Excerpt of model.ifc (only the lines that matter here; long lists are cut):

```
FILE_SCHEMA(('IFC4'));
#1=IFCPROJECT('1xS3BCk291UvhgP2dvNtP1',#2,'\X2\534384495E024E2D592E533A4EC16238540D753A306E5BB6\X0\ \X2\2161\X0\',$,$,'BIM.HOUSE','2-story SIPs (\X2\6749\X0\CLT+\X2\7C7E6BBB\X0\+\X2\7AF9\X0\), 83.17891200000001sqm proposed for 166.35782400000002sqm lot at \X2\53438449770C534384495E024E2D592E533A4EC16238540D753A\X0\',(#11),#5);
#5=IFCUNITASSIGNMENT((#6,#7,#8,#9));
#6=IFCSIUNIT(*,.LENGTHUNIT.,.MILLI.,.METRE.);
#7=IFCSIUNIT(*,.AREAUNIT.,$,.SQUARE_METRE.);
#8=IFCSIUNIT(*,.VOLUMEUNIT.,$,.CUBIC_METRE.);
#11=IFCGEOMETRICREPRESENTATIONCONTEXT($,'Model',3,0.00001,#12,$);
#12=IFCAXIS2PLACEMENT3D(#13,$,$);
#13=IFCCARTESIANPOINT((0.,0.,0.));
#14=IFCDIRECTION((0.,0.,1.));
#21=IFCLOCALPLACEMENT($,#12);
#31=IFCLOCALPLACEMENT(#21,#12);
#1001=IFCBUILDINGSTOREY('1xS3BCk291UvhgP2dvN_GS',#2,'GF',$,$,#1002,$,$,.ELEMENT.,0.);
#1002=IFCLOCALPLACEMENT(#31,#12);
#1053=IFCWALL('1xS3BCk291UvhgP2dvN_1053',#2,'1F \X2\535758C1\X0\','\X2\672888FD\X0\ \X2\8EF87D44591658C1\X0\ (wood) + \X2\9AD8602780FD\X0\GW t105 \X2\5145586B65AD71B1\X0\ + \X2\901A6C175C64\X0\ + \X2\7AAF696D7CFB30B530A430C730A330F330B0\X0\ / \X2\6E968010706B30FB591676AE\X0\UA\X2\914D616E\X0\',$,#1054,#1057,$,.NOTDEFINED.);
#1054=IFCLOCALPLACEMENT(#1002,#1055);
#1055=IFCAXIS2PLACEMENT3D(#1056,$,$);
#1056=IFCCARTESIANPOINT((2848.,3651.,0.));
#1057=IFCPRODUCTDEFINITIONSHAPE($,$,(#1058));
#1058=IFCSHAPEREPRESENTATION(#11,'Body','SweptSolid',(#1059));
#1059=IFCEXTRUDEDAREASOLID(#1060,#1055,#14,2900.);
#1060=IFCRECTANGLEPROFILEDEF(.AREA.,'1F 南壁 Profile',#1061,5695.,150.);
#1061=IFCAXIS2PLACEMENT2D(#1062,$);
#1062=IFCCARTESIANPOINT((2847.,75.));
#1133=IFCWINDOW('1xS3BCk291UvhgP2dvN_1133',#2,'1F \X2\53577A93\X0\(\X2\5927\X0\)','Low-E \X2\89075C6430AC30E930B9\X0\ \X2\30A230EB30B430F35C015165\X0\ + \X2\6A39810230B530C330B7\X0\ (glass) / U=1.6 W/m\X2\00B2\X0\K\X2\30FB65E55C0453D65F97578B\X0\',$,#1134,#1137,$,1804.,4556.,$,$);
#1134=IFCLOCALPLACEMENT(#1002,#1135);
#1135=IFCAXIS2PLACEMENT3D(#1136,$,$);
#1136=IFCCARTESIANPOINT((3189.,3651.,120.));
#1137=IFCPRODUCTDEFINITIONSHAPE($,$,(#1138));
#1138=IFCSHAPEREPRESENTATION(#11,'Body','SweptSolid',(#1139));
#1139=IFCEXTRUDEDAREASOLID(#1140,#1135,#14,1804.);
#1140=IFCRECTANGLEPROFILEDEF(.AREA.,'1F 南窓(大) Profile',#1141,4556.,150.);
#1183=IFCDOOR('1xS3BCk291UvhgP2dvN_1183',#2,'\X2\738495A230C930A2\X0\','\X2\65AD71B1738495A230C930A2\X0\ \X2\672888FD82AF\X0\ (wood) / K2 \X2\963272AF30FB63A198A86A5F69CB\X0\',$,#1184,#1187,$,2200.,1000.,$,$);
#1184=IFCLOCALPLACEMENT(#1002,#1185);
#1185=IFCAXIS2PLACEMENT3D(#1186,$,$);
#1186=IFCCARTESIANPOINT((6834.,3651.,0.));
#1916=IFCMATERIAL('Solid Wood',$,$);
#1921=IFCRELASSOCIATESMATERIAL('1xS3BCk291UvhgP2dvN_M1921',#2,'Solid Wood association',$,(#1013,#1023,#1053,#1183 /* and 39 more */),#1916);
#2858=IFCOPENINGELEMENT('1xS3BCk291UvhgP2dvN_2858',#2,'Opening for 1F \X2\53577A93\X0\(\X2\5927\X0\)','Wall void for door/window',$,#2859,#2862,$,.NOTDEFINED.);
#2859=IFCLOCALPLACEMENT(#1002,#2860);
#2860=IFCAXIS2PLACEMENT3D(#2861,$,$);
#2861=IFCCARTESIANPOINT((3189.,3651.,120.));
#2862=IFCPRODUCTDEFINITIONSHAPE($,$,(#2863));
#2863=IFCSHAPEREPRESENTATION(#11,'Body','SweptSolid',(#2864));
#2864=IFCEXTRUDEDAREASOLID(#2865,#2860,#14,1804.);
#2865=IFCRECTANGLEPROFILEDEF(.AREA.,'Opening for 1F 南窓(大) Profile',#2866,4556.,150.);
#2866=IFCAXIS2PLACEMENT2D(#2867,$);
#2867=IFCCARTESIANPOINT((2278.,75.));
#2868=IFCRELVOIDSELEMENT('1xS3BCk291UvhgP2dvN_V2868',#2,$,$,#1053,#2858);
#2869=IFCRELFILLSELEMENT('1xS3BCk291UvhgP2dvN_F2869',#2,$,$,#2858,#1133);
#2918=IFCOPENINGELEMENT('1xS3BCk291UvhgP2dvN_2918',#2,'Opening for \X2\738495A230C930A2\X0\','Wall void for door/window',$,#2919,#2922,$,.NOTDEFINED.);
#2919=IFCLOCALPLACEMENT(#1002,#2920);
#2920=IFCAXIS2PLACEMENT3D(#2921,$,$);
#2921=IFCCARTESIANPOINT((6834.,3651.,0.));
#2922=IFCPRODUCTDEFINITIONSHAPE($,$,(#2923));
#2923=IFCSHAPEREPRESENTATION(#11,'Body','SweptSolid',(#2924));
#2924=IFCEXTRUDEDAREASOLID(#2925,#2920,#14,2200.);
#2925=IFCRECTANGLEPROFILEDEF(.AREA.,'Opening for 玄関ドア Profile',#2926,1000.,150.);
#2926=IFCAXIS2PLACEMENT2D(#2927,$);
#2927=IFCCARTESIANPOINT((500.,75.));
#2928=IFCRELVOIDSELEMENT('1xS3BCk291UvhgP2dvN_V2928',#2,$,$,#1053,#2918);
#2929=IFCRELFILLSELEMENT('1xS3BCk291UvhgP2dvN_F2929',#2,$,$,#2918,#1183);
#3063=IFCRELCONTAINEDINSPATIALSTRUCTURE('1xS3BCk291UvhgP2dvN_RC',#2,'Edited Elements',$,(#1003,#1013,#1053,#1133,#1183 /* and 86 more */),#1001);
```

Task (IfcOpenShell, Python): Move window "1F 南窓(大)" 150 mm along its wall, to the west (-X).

```python
import ifcopenshell
import ifcopenshell.api.geometry
import ifcopenshell.util.placement
import ifcopenshell.util.unit

model = ifcopenshell.open("model.ifc")
unit_scale = ifcopenshell.util.unit.calculate_unit_scale(model)

window = model.by_guid("1xS3BCk291UvhgP2dvN_1133")
opening = window.FillsVoids[0].RelatingOpeningElement
wall = opening.VoidsElements[0].RelatingBuildingElement

wall_matrix = ifcopenshell.util.placement.get_local_placement(wall.ObjectPlacement)
shift = wall_matrix[:3, 0] * -0.15 / unit_scale
before = ifcopenshell.util.placement.get_local_placement(window.ObjectPlacement)[:3, 3].copy()

# The window is not placed relative to its opening, so move both.
for product in (opening, window):
    matrix = ifcopenshell.util.placement.get_local_placement(product.ObjectPlacement)
    matrix[:3, 3] += shift
    ifcopenshell.api.geometry.edit_object_placement(model, product=product, matrix=matrix, is_si=False)

after = ifcopenshell.util.placement.get_local_placement(window.ObjectPlacement)[:3, 3]
print("window moved by", (after - before).round(3) + 0.0)

model.write("model_v2.ifc")
```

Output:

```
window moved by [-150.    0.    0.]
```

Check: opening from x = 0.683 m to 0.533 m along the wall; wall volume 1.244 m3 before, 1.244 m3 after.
